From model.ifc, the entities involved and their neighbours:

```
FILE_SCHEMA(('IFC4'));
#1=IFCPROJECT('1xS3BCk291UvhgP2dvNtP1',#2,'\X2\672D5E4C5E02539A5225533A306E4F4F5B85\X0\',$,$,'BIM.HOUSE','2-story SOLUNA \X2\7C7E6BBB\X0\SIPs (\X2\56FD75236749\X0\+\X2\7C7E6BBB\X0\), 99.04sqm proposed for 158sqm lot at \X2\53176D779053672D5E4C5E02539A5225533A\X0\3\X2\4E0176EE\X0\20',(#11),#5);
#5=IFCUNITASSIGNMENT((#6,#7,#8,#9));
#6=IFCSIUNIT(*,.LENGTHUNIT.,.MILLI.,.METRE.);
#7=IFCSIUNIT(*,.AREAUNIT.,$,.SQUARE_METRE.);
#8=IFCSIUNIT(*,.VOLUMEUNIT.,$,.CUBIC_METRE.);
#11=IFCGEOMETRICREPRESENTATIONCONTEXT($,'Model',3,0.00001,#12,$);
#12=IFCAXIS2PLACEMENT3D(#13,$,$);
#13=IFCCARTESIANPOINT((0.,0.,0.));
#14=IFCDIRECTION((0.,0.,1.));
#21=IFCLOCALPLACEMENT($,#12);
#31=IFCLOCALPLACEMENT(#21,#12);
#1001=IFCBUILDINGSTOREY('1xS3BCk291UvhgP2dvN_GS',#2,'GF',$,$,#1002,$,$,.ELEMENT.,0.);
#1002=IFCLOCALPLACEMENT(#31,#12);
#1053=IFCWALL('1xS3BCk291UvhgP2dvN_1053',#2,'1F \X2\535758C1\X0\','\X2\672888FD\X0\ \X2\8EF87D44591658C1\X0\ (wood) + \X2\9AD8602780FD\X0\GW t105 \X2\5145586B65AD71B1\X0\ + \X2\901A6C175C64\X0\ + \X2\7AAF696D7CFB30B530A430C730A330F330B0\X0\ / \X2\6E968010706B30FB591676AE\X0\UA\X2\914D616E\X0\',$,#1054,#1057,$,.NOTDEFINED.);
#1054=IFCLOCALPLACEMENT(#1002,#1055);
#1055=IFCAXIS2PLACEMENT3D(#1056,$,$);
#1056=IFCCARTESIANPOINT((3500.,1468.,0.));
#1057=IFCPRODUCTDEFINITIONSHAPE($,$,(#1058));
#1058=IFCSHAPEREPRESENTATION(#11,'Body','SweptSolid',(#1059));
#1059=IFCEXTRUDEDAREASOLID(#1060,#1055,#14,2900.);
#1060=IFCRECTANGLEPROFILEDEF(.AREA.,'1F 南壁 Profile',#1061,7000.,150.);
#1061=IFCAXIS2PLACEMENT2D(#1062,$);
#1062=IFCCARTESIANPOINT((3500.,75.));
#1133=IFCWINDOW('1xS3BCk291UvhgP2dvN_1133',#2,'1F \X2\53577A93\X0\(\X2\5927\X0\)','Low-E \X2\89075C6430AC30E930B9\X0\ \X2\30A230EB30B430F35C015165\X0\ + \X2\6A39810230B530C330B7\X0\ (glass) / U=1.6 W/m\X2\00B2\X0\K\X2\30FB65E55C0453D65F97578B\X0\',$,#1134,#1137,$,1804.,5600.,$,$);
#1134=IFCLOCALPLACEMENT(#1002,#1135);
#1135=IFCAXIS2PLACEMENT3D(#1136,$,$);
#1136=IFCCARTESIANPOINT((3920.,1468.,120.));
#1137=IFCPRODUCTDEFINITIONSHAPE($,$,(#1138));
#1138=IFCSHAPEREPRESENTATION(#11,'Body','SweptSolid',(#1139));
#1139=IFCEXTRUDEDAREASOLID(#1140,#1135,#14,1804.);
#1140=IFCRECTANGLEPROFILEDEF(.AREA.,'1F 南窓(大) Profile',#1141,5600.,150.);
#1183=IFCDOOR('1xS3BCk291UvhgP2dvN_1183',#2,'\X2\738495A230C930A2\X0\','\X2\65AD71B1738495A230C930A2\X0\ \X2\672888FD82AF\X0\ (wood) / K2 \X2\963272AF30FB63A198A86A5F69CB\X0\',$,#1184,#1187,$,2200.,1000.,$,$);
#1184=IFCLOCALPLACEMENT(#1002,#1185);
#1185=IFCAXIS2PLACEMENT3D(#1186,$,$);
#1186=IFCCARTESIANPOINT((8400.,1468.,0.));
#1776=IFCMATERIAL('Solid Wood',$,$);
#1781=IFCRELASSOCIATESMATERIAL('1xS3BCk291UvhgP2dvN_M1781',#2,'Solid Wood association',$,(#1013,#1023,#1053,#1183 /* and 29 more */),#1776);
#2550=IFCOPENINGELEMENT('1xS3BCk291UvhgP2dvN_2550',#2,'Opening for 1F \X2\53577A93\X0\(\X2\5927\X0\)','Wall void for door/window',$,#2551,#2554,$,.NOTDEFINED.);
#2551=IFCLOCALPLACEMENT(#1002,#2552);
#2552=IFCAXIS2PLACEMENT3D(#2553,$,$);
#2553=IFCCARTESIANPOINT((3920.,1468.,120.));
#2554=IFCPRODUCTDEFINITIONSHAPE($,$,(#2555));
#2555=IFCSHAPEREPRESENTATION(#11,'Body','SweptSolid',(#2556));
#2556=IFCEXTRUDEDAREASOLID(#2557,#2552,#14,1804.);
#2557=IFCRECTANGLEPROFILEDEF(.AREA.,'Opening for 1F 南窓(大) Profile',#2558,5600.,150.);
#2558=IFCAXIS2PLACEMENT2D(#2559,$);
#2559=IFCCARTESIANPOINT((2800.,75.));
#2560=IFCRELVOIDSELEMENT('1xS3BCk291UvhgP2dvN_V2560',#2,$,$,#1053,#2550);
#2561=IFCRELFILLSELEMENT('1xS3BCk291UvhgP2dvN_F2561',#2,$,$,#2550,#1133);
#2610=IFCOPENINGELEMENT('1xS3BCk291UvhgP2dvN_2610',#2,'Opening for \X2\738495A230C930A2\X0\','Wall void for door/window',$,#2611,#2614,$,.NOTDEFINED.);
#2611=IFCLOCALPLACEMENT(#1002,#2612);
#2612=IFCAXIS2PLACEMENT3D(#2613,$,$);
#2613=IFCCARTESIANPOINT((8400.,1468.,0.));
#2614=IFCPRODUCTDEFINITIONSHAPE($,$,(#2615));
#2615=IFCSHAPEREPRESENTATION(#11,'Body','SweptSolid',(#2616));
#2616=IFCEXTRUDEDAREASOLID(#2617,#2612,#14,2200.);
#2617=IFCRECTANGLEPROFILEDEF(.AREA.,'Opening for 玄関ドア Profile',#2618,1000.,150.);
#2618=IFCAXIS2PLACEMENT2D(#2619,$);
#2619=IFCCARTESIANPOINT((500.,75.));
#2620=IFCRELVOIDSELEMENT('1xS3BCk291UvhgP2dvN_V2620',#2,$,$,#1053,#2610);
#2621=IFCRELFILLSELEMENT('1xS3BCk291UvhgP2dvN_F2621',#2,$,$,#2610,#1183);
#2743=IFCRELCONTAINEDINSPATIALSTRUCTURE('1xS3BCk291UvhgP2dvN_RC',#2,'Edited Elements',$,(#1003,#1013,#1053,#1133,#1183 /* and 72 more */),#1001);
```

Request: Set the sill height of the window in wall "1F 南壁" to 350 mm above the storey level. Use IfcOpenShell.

```python
import numpy as np
import ifcopenshell
import ifcopenshell.api.geometry
import ifcopenshell.geom
import ifcopenshell.util.element
import ifcopenshell.util.placement
import ifcopenshell.util.shape
import ifcopenshell.util.unit

model = ifcopenshell.open("model.ifc")
unit_scale = ifcopenshell.util.unit.calculate_unit_scale(model)

window = model.by_guid("1xS3BCk291UvhgP2dvN_1133")
opening = window.FillsVoids[0].RelatingOpeningElement
storey = ifcopenshell.util.element.get_container(window, ifc_class="IfcBuildingStorey")
level = ifcopenshell.util.placement.get_local_placement(storey.ObjectPlacement)[2, 3]

# The opening's origin need not be at the sill, so measure its lowest point.
shape = ifcopenshell.geom.create_shape(ifcopenshell.geom.settings(), opening)
bottom = ifcopenshell.util.shape.get_shape_bottom_elevation(shape, shape.geometry) / unit_scale
dz = level + 350.0 - bottom

shift = np.array([0.0, 0.0, dz])
# The window is not placed relative to its opening, so move both.
for product in (opening, window):
    matrix = ifcopenshell.util.placement.get_local_placement(product.ObjectPlacement)
    matrix[:3, 3] += shift
    ifcopenshell.api.geometry.edit_object_placement(model, product=product, matrix=matrix, is_si=False)

print(f"moved by {dz * unit_scale:+.3f} m")

model.write("model_rev.ifc")
```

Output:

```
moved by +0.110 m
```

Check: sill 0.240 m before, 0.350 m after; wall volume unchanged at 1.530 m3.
